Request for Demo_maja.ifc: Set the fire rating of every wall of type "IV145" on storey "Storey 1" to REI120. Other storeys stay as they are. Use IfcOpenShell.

First a look at what the model holds.

```python
import ifcopenshell
import ifcopenshell.util.element

model = ifcopenshell.open("Demo_maja.ifc")
print(model.schema)
storey = next(s for s in model.by_type("IfcBuildingStorey") if s.Name == "Storey 1")
walls = [e for e in ifcopenshell.util.element.get_decomposition(storey) if e.is_a("IfcWall")]
seen = {}
for e in walls:
    element_type = ifcopenshell.util.element.get_type(e)
    key = (element_type.Name if element_type != e and element_type else None, ifcopenshell.util.element.get_pset(e, "Pset_WallCommon", "FireRating"))
    seen[key] = seen.get(key, 0) + 1
for (name, value), count in sorted(seen.items(), key=str):
    print(count, "x", name, "|", value)
```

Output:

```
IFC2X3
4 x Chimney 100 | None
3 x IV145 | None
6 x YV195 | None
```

```python
import ifcopenshell
import ifcopenshell.api.pset
import ifcopenshell.util.element

model = ifcopenshell.open("Demo_maja.ifc")

storey = next(s for s in model.by_type("IfcBuildingStorey") if s.Name == "Storey 1")
walls = [e for e in ifcopenshell.util.element.get_decomposition(storey) if e.is_a("IfcWall")]

count = 0
for e in walls:
    element_type = ifcopenshell.util.element.get_type(e)
    if element_type in (None, e) or element_type.Name != "IV145":
        continue
    # add_pset returns the element's existing set when there is one.
    pset = ifcopenshell.api.pset.add_pset(model, product=e, name="Pset_WallCommon")
    ifcopenshell.api.pset.edit_pset(model, pset=pset, properties={"FireRating": "REI120"})
    count += 1

print(count, "walls updated")

model.write("Demo_maja_rev.ifc")
```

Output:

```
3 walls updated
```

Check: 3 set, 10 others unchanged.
